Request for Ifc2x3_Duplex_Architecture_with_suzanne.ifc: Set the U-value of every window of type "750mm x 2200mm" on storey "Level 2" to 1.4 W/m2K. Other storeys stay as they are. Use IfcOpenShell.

First a look at what the model holds.

```python
import ifcopenshell
import ifcopenshell.util.element

model = ifcopenshell.open("Ifc2x3_Duplex_Architecture_with_suzanne.ifc")
print(model.schema)
storey = next(s for s in model.by_type("IfcBuildingStorey") if s.Name == "Level 2")
windows = [e for e in ifcopenshell.util.element.get_decomposition(storey) if e.is_a("IfcWindow")]
seen = {}
for e in windows:
    element_type = ifcopenshell.util.element.get_type(e)
    key = (element_type.Name if element_type != e and element_type else None, ifcopenshell.util.element.get_pset(e, "Pset_WindowCommon", "ThermalTransmittance"))
    seen[key] = seen.get(key, 0) + 1
for (name, value), count in sorted(seen.items(), key=str):
    print(count, "x", name, "|", value)
```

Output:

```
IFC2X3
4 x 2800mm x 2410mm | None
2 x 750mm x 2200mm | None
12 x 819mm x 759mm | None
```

```python
import ifcopenshell
import ifcopenshell.api.pset
import ifcopenshell.util.element

model = ifcopenshell.open("Ifc2x3_Duplex_Architecture_with_suzanne.ifc")

storey = next(s for s in model.by_type("IfcBuildingStorey") if s.Name == "Level 2")
windows = [e for e in ifcopenshell.util.element.get_decomposition(storey) if e.is_a("IfcWindow")]

count = 0
for e in windows:
    element_type = ifcopenshell.util.element.get_type(e)
    if element_type in (None, e) or element_type.Name != "750mm x 2200mm":
        continue
    # add_pset returns the element's existing set when there is one.
    pset = ifcopenshell.api.pset.add_pset(model, product=e, name="Pset_WindowCommon")
    ifcopenshell.api.pset.edit_pset(model, pset=pset, properties={"ThermalTransmittance": 1.4})
    count += 1

print(count, "windows updated")

model.write("Ifc2x3_Duplex_Architecture_with_suzanne_rev.ifc")
```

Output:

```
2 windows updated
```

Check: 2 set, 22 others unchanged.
